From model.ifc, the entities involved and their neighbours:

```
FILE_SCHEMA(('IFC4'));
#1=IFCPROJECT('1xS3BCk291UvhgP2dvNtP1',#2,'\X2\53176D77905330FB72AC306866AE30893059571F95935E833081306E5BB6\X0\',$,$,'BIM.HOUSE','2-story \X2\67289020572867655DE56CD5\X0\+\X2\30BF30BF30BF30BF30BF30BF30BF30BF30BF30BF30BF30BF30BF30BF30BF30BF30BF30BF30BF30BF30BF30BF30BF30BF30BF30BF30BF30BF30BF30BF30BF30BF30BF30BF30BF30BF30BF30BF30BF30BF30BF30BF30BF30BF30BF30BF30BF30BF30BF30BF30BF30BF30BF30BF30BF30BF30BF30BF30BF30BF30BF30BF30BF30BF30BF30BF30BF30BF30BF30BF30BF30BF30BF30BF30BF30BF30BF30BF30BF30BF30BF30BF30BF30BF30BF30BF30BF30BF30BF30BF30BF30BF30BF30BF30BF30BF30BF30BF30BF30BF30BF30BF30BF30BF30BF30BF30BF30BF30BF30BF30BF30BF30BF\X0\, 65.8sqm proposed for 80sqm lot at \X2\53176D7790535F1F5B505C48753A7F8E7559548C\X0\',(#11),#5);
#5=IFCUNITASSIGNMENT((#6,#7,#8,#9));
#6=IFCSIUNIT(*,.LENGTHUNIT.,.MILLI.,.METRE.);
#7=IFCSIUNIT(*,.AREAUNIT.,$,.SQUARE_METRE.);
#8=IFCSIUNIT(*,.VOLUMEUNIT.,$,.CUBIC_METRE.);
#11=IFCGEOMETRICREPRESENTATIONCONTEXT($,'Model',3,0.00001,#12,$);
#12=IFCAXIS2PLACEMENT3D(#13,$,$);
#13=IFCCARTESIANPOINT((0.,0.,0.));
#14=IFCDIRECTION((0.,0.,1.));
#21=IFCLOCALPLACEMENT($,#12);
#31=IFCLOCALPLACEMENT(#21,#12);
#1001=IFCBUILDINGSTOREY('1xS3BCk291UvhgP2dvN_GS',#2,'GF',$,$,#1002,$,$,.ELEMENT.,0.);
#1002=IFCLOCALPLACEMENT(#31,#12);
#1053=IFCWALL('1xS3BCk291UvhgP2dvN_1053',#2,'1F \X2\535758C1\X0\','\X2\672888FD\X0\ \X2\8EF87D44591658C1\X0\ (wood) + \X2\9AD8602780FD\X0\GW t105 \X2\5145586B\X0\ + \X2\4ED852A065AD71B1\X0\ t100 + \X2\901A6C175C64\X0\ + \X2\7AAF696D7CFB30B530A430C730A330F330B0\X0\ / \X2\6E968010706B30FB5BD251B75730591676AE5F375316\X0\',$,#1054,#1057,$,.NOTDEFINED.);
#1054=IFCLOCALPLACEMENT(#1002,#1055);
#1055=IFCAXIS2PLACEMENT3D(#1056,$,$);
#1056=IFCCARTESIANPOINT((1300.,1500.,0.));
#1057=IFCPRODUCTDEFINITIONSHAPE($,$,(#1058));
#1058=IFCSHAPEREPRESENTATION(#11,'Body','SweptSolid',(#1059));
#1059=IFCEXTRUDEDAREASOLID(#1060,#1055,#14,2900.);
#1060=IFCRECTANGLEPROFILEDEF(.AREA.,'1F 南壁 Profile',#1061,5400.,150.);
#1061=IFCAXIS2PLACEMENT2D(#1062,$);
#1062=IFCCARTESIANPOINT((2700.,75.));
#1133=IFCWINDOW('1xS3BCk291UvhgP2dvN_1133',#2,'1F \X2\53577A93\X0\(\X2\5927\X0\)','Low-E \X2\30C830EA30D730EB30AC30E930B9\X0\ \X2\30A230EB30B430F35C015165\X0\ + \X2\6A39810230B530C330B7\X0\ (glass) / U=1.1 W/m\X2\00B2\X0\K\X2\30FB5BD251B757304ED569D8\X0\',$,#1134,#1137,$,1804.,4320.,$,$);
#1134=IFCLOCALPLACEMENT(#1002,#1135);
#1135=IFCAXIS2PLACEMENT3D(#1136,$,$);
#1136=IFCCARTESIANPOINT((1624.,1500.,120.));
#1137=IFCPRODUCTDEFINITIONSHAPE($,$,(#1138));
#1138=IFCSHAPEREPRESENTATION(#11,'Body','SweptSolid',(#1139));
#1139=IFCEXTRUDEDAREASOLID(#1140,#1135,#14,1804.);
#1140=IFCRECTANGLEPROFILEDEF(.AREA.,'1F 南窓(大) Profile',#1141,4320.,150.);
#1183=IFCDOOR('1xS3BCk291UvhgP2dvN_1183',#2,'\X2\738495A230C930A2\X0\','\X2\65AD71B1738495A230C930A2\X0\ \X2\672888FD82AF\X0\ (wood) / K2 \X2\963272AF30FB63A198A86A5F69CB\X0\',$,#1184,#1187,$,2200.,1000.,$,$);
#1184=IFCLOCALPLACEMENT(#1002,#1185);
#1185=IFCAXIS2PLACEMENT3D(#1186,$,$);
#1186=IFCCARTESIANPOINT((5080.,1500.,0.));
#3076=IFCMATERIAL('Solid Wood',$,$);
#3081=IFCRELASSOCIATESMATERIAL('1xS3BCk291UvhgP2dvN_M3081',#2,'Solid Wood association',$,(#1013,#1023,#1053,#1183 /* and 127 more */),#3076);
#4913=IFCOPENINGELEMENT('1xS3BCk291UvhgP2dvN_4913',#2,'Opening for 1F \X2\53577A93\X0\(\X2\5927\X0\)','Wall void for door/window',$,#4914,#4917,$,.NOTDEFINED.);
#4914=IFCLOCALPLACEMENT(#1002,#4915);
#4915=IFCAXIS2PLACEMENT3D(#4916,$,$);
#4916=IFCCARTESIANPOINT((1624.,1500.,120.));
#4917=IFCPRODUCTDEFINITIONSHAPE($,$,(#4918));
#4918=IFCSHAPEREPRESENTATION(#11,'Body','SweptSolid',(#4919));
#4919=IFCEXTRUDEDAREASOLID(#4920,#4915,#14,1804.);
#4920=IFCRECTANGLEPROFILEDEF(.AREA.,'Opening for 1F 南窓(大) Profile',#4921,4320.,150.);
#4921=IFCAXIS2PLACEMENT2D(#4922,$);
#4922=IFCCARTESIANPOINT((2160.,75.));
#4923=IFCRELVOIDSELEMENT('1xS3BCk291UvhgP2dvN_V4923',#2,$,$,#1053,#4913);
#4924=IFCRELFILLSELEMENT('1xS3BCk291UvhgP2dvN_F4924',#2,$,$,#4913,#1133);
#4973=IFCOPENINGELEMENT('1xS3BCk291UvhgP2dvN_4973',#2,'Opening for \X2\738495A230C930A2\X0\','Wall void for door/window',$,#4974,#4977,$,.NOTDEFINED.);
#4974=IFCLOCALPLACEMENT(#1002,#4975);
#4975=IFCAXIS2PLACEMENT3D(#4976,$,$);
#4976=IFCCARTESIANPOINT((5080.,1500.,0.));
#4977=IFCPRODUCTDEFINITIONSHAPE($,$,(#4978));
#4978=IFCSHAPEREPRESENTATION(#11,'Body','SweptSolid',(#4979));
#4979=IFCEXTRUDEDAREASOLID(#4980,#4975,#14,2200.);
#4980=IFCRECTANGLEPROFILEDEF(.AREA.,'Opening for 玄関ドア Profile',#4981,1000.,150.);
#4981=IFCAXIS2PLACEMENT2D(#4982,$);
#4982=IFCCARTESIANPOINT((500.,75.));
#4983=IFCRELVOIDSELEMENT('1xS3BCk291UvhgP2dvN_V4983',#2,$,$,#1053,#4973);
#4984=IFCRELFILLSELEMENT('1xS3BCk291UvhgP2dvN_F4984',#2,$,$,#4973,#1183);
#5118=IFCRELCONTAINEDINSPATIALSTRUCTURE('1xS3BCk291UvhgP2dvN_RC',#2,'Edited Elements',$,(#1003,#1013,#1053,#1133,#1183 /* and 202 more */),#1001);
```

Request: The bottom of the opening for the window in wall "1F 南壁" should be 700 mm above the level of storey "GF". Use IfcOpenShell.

```python
import numpy as np
import ifcopenshell
import ifcopenshell.api.geometry
import ifcopenshell.geom
import ifcopenshell.util.element
import ifcopenshell.util.placement
import ifcopenshell.util.shape
import ifcopenshell.util.unit

model = ifcopenshell.open("model.ifc")
unit_scale = ifcopenshell.util.unit.calculate_unit_scale(model)

window = model.by_guid("1xS3BCk291UvhgP2dvN_1133")
opening = window.FillsVoids[0].RelatingOpeningElement
storey = ifcopenshell.util.element.get_container(window, ifc_class="IfcBuildingStorey")
level = ifcopenshell.util.placement.get_local_placement(storey.ObjectPlacement)[2, 3]

# The opening's origin need not be at the sill, so measure its lowest point.
shape = ifcopenshell.geom.create_shape(ifcopenshell.geom.settings(), opening)
bottom = ifcopenshell.util.shape.get_shape_bottom_elevation(shape, shape.geometry) / unit_scale
dz = level + 700.0 - bottom

shift = np.array([0.0, 0.0, dz])
# The window is not placed relative to its opening, so move both.
for product in (opening, window):
    matrix = ifcopenshell.util.placement.get_local_placement(product.ObjectPlacement)
    matrix[:3, 3] += shift
    ifcopenshell.api.geometry.edit_object_placement(model, product=product, matrix=matrix, is_si=False)

print(f"moved by {dz * unit_scale:+.3f} m")

model.write("model_updated.ifc")
```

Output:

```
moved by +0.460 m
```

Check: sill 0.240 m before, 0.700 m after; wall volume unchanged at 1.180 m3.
